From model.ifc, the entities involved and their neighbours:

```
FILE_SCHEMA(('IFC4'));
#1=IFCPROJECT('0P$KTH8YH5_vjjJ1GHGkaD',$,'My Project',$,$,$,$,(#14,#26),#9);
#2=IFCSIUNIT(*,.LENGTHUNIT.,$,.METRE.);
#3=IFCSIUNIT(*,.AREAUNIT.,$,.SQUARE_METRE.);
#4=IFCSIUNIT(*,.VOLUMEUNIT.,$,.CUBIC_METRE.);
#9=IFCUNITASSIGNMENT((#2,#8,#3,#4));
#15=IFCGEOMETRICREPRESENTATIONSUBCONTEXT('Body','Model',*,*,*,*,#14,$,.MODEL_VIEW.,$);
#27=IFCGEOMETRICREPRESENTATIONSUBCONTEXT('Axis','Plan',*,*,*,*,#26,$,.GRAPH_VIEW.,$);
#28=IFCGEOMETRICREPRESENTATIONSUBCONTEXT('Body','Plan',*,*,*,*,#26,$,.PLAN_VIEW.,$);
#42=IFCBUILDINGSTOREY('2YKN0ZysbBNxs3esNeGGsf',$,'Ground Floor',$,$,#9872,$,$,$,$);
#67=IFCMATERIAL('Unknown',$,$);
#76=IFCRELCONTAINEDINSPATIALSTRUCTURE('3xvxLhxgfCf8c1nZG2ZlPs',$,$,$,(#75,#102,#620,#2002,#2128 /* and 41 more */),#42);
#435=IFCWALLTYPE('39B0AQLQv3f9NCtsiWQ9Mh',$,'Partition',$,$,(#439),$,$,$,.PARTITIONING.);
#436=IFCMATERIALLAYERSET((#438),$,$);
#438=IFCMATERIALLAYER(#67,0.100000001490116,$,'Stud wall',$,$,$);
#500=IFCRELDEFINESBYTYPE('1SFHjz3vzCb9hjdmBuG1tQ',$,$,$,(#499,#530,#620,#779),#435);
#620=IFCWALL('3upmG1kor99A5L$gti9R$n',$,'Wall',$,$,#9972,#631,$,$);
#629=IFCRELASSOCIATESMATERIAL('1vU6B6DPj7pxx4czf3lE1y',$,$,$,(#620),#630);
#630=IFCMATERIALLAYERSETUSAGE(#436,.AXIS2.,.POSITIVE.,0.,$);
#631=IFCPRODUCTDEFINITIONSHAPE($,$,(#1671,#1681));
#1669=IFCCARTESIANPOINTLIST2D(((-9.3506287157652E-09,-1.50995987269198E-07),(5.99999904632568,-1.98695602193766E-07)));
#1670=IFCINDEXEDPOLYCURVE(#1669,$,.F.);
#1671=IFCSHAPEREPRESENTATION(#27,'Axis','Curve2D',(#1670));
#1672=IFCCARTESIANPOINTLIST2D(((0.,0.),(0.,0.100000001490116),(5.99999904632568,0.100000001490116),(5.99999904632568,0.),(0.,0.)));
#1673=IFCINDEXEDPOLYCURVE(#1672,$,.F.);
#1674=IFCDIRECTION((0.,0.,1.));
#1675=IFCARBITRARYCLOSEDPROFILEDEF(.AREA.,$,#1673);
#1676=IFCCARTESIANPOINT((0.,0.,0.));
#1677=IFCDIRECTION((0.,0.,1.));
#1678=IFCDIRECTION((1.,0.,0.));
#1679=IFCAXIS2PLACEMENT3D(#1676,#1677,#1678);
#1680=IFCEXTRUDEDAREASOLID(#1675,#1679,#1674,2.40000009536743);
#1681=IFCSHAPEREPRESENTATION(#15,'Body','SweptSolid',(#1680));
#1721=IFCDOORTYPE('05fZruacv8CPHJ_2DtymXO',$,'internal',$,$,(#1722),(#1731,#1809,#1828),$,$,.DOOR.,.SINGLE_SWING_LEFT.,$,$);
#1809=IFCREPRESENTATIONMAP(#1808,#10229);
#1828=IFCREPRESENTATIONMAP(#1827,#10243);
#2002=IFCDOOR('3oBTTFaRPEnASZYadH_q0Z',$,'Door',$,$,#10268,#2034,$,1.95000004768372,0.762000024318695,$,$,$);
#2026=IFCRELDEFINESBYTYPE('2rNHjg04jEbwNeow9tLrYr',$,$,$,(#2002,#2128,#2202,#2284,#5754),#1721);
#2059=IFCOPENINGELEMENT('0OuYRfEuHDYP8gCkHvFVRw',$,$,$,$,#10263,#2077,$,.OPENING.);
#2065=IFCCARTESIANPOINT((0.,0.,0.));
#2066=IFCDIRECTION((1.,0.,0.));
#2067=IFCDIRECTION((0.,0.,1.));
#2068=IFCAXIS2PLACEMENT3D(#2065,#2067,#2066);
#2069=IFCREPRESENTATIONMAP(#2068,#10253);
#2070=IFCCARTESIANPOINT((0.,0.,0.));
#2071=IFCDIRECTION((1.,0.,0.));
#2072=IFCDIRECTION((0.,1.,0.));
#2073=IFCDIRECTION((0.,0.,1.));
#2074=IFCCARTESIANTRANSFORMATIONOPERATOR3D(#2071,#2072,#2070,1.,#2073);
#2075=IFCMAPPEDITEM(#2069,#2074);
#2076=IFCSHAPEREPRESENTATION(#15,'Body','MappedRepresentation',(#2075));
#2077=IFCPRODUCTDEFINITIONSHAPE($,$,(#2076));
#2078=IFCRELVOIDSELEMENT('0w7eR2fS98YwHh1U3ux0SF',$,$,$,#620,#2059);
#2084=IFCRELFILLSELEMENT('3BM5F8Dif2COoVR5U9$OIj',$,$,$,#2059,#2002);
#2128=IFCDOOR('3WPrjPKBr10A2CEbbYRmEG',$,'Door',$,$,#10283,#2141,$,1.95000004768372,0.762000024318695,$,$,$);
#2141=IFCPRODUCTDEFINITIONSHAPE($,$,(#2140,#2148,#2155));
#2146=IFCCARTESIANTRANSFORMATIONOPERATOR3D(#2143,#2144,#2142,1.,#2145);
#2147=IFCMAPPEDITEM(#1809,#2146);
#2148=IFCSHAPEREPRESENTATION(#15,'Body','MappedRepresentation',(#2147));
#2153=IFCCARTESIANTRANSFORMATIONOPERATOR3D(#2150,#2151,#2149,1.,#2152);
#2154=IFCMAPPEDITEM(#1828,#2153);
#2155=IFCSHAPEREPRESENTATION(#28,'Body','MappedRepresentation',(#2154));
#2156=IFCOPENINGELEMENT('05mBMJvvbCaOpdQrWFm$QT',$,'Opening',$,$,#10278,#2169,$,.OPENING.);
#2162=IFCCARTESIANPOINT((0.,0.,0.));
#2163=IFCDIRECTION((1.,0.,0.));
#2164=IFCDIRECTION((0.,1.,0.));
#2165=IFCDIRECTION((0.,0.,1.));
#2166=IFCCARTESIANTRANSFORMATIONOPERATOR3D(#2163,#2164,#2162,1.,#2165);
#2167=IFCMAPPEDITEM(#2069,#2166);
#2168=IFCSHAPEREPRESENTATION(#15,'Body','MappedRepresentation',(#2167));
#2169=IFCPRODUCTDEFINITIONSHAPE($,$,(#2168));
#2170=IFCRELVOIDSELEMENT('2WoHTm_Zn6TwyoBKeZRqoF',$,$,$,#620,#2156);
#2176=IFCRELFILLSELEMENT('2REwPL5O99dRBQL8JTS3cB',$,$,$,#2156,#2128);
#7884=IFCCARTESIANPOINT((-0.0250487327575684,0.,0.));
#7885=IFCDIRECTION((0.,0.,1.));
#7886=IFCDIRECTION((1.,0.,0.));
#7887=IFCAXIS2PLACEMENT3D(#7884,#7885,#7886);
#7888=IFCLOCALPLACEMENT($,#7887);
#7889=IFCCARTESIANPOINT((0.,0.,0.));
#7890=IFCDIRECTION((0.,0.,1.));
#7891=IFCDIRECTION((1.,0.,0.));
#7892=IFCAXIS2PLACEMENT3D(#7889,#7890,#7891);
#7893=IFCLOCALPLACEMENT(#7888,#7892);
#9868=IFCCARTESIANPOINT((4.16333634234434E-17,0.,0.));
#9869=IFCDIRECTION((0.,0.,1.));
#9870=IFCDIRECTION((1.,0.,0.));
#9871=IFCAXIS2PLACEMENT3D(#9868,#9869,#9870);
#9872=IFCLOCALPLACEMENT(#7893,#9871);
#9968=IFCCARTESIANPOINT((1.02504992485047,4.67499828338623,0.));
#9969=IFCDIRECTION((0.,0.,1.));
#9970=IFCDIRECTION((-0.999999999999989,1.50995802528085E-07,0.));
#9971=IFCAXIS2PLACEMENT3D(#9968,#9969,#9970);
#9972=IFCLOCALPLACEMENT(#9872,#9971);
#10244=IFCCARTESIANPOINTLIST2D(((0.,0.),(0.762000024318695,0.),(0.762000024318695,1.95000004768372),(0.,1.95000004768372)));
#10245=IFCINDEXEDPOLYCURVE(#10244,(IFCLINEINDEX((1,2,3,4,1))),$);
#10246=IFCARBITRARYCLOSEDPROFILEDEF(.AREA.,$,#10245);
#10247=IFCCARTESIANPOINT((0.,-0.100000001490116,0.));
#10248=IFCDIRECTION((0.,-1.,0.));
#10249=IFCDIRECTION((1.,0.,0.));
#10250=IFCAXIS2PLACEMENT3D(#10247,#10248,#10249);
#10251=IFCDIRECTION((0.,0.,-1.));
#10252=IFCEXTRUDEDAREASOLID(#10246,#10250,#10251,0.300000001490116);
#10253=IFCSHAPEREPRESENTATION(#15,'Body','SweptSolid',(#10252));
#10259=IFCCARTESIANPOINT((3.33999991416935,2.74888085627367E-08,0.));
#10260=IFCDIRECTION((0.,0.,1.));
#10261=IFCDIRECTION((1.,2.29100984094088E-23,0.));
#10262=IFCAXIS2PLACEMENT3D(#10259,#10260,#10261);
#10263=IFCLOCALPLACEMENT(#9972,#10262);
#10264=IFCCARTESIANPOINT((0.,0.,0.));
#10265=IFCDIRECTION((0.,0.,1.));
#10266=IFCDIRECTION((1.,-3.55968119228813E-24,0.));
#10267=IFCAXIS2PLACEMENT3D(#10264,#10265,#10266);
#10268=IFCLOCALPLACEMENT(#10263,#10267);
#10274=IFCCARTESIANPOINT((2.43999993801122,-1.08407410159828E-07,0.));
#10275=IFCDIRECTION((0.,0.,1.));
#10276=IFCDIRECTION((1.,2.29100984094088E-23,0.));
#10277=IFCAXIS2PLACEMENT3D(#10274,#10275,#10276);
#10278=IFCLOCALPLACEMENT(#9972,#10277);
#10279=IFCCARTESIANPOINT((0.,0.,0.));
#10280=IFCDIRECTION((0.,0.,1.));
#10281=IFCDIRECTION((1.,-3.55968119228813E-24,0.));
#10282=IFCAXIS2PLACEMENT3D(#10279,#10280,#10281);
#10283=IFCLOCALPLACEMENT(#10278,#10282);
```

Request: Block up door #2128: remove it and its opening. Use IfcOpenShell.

```python
import ifcopenshell
import ifcopenshell.api.feature
import ifcopenshell.api.root
import ifcopenshell.geom
import ifcopenshell.util.shape

model = ifcopenshell.open("model.ifc")
settings = ifcopenshell.geom.settings()


def volume(element):
    """Net volume in cubic metres, openings subtracted."""
    shape = ifcopenshell.geom.create_shape(settings, element)
    return ifcopenshell.util.shape.get_volume(shape.geometry)


door = model.by_id(2128)
opening = door.FillsVoids[0].RelatingOpeningElement
wall = opening.VoidsElements[0].RelatingBuildingElement
before = volume(wall)

ifcopenshell.api.root.remove_product(model, product=door)
ifcopenshell.api.feature.remove_feature(model, feature=opening)

after = volume(wall)

print(f"wall volume {before:.3f} -> {after:.3f} m3")

model.write("model_updated.ifc")
```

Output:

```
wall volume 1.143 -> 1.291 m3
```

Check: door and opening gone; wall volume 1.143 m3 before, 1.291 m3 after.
